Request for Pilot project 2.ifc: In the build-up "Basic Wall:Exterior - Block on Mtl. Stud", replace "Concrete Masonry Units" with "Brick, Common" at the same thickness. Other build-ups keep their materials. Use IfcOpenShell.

First a look at what the model holds.

```python
import ifcopenshell
import ifcopenshell.util.element

model = ifcopenshell.open("Pilot project 2.ifc")
print(model.schema)
for layer_set in model.by_type("IfcMaterialLayerSet"):
    if layer_set.LayerSetName == "Basic Wall:Exterior - Block on Mtl. Stud":
        for layer in layer_set.MaterialLayers:
            print(layer.id(), layer.Material and layer.Material.Name, layer.LayerThickness, sep=" | ")
        print(len(ifcopenshell.util.element.get_elements_by_material(model, layer_set)), "elements and types use it")
print(sorted(m.Name for m in model.by_type("IfcMaterial") if m.Name)[:60])
```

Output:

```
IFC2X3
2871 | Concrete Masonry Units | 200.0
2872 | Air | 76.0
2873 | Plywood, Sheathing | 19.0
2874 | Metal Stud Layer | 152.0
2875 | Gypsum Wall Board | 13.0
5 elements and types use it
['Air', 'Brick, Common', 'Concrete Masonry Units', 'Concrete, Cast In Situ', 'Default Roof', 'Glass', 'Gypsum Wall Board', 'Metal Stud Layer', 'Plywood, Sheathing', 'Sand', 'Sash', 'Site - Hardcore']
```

```python
import ifcopenshell
import ifcopenshell.api.material

model = ifcopenshell.open("Pilot project 2.ifc")

layer_set = next(s for s in model.by_type("IfcMaterialLayerSet") if s.LayerSetName == "Basic Wall:Exterior - Block on Mtl. Stud")
layer = next(l for l in layer_set.MaterialLayers if l.Material and l.Material.Name == "Concrete Masonry Units")
material = next(m for m in model.by_type("IfcMaterial") if m.Name == "Brick, Common")

# Point this one layer at the other material; renaming the old one would change it everywhere.
ifcopenshell.api.material.edit_layer(model, layer=layer, attributes={}, material=material)

print([l.Material.Name if l.Material else None for l in layer_set.MaterialLayers])

model.write("Pilot project 2-out.ifc")
```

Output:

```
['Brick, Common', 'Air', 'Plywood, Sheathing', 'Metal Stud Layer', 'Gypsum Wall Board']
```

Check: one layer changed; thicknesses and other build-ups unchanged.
